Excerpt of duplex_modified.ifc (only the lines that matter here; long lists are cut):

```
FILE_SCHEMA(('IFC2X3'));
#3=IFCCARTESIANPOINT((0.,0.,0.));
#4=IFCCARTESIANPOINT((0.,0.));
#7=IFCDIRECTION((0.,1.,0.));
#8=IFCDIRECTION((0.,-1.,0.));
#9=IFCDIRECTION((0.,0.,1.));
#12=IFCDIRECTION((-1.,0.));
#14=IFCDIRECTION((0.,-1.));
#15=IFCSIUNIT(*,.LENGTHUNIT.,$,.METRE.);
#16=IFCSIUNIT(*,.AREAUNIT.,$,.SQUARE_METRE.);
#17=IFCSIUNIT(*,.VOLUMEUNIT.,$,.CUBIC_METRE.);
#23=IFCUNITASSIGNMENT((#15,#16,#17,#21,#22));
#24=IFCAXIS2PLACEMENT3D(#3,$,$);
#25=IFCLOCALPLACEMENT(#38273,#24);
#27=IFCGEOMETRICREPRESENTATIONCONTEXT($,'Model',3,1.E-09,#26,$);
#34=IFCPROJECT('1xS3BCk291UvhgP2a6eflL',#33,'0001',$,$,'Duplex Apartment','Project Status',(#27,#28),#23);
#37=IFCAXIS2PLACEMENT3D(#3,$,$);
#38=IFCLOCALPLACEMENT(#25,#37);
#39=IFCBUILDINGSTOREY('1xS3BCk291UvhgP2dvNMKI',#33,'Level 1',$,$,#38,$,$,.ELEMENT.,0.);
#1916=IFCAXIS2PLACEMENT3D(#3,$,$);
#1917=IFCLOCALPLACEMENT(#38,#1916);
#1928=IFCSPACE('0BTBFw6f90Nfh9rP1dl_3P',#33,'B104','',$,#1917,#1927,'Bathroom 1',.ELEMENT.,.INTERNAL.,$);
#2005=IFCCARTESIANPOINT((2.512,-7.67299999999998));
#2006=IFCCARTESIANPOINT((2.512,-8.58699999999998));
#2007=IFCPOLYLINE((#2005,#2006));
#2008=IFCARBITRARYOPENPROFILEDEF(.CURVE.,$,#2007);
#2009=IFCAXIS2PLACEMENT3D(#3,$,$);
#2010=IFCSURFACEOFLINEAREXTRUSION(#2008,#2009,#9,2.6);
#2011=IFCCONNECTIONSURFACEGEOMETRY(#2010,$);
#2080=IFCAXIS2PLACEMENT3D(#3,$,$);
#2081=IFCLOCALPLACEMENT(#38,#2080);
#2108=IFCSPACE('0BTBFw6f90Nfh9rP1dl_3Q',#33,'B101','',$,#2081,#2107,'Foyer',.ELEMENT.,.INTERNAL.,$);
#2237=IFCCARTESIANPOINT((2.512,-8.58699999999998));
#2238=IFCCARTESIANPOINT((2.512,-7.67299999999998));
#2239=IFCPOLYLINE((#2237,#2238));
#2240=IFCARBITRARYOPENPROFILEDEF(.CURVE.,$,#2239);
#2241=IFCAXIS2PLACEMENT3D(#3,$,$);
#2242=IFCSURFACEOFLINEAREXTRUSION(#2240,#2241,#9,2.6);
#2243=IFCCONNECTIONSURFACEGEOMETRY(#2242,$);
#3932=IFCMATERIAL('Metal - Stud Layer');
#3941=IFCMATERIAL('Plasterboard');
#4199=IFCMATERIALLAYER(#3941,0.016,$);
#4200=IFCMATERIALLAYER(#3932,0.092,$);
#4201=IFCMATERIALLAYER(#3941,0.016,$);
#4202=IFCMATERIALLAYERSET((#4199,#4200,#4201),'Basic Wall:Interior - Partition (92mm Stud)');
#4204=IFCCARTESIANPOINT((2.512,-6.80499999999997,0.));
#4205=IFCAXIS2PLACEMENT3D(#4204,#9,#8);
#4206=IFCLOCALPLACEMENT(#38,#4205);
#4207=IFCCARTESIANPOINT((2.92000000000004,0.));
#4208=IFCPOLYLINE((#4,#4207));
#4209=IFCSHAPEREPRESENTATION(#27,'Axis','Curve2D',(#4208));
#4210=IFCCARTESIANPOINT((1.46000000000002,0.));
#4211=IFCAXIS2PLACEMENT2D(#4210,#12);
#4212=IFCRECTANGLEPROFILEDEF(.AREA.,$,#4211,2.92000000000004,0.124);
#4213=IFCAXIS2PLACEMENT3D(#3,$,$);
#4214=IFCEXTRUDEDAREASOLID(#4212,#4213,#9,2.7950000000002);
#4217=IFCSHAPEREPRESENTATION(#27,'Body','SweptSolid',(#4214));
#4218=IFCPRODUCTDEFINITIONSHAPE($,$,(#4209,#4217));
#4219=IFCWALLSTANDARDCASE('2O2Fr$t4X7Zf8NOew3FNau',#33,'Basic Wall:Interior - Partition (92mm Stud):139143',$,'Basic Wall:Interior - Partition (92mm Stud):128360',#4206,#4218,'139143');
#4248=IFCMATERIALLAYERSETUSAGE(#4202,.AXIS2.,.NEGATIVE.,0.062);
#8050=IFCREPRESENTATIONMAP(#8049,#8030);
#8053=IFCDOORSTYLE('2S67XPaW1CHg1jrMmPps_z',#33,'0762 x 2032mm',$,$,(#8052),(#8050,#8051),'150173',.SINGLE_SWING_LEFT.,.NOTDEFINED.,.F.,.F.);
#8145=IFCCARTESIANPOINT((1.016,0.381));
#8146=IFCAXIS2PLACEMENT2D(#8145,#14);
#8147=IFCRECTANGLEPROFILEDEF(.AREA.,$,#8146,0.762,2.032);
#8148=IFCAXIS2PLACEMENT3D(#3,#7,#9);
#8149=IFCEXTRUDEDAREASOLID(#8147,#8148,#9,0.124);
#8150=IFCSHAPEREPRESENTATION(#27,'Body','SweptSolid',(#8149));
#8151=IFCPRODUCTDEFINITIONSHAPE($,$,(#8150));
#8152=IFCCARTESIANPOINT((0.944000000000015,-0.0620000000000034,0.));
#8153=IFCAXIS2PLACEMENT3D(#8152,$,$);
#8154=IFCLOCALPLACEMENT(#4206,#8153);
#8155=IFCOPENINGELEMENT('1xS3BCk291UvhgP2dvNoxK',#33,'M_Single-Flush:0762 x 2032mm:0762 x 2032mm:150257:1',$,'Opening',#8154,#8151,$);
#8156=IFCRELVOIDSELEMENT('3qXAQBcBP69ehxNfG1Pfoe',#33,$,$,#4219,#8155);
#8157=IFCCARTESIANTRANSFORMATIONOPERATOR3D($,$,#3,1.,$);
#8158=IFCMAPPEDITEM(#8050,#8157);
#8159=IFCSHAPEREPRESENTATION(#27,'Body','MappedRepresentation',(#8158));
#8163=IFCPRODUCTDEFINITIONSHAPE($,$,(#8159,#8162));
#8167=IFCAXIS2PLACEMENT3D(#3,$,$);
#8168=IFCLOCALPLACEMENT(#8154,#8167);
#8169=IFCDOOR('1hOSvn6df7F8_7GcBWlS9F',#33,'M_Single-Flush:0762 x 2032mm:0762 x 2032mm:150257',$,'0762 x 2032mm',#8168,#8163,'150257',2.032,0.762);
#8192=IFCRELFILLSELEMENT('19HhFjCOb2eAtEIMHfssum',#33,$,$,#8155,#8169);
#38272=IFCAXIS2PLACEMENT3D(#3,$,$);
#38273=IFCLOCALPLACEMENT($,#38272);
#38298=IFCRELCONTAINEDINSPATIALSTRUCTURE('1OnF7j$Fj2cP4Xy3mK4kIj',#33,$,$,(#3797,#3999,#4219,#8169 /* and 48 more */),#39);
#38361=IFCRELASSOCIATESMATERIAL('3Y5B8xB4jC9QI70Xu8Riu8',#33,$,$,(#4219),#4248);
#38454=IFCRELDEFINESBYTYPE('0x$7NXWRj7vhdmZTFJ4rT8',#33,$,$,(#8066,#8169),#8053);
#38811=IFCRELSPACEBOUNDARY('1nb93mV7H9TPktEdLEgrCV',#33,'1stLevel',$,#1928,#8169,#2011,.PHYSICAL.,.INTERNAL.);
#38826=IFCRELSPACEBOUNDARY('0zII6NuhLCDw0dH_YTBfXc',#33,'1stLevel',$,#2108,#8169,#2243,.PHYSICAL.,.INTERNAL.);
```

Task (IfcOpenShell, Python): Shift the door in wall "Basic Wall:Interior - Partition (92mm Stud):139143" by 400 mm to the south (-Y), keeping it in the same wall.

```python
import numpy as np
import ifcopenshell
import ifcopenshell.api.geometry
import ifcopenshell.util.placement
import ifcopenshell.util.unit

model = ifcopenshell.open("duplex_modified.ifc")
unit_scale = ifcopenshell.util.unit.calculate_unit_scale(model)

door = model.by_id(8169)
opening = door.FillsVoids[0].RelatingOpeningElement
wall = opening.VoidsElements[0].RelatingBuildingElement

wall_matrix = ifcopenshell.util.placement.get_local_placement(wall.ObjectPlacement)
shift = wall_matrix[:3, 0] * 0.4 / unit_scale
before = ifcopenshell.util.placement.get_local_placement(door.ObjectPlacement)[:3, 3].copy()

# The door is placed relative to its opening, so it follows when the opening moves.
matrix = ifcopenshell.util.placement.get_local_placement(opening.ObjectPlacement)
matrix[:3, 3] += shift
ifcopenshell.api.geometry.edit_object_placement(
    model, product=opening, matrix=matrix, is_si=False, should_transform_children=True
)

# Space boundary surfaces are stored in each space's coordinates; move them too.
for rel in door.ProvidesBoundaries:
    if not rel.ConnectionGeometry:
        continue
    surface = rel.ConnectionGeometry.SurfaceOnRelatingElement
    space_matrix = ifcopenshell.util.placement.get_local_placement(rel.RelatingSpace.ObjectPlacement)
    point = np.array(surface.Position.Location.Coordinates) + space_matrix[:3, :3].T @ shift
    surface.Position = model.createIfcAxis2Placement3D(
        model.createIfcCartesianPoint(point.tolist()), surface.Position.Axis, surface.Position.RefDirection
    )

after = ifcopenshell.util.placement.get_local_placement(door.ObjectPlacement)[:3, 3]
print("door moved by", (after - before).round(3) + 0.0)

model.write("duplex_modified_v2.ifc")
```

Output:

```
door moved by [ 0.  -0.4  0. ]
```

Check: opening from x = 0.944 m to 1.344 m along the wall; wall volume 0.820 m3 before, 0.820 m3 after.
